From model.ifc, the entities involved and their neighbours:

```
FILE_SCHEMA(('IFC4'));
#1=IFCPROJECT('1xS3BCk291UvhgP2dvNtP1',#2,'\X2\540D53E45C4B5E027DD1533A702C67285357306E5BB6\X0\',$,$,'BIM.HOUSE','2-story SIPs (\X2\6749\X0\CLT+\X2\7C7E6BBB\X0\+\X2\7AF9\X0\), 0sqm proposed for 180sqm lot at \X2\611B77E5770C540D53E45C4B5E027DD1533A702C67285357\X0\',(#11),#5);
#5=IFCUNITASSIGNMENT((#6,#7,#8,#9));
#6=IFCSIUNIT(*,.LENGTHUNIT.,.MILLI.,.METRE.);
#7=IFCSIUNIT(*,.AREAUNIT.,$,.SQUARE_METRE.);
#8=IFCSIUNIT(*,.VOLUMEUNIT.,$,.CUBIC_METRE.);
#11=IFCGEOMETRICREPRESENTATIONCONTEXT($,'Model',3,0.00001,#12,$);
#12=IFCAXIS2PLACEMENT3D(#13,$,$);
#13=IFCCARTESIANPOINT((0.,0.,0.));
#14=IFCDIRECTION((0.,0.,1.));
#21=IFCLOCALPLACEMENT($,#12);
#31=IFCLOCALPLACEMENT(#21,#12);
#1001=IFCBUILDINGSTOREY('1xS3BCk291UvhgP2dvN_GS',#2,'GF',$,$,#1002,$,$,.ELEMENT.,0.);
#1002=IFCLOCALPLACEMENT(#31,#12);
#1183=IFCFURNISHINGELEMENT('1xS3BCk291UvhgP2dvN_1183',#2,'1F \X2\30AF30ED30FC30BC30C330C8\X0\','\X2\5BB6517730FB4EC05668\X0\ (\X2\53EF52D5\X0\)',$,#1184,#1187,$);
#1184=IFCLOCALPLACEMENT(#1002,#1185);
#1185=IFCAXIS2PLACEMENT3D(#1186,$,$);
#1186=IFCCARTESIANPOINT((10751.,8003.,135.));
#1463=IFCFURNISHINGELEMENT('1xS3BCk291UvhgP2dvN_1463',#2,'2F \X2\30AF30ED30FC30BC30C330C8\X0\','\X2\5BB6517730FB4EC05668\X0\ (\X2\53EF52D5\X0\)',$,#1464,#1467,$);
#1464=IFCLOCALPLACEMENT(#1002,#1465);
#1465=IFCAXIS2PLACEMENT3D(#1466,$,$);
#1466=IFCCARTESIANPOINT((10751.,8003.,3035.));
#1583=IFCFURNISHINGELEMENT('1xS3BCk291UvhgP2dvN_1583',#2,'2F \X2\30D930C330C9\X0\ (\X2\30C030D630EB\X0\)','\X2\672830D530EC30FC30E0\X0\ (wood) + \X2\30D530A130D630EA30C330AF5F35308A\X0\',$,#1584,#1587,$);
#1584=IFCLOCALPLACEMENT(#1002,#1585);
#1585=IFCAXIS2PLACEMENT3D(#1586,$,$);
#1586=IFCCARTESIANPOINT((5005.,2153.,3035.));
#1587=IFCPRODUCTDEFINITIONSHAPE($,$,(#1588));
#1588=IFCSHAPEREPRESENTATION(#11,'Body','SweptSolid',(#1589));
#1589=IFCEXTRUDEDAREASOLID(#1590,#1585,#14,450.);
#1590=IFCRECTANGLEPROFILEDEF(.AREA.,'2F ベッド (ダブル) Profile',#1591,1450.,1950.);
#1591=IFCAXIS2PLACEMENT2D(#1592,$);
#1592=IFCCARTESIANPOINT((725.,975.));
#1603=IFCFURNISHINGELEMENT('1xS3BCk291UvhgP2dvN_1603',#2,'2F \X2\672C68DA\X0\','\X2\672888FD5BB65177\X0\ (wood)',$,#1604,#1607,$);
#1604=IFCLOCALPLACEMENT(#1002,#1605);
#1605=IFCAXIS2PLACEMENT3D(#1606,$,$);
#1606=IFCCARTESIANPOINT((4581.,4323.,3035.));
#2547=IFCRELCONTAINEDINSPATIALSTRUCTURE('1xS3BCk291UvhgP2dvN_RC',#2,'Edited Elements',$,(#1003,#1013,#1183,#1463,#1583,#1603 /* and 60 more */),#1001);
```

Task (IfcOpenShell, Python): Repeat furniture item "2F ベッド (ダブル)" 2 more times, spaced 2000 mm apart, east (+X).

```python
import numpy as np
import ifcopenshell
import ifcopenshell.api.geometry
import ifcopenshell.api.root
import ifcopenshell.util.element
import ifcopenshell.util.placement

model = ifcopenshell.open("model.ifc")


def reuse_history(source, copy):
    """copy_class also copies each property set's owner history, people and application; keep the originals."""
    for rel in copy.IsDefinedBy:
        if rel.is_a("IfcRelDefinesByProperties") and (history := rel.RelatingPropertyDefinition.OwnerHistory):
            rel.RelatingPropertyDefinition.OwnerHistory = source.OwnerHistory
            ifcopenshell.util.element.remove_deep2(model, history)


source = model.by_guid("1xS3BCk291UvhgP2dvN_1583")
base = ifcopenshell.util.placement.get_local_placement(source.ObjectPlacement)
step = np.array([1.0, 0.0, 0.0]) * 2000.0

for i in range(1, 3):
    copy = ifcopenshell.api.root.copy_class(model, product=source)
    copy.Representation = ifcopenshell.util.element.copy_deep(
        model, source.Representation, exclude=["IfcGeometricRepresentationContext", "IfcRepresentationMap"]
    )
    reuse_history(source, copy)
    matrix = base.copy()
    matrix[:3, 3] += i * step
    print("added at", matrix[:3, 3].round(3) + 0.0)
    ifcopenshell.api.geometry.edit_object_placement(model, product=copy, matrix=matrix, is_si=False)

model.write("model_v2.ifc")
```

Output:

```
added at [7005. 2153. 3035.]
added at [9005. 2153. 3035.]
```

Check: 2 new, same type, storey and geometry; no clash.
